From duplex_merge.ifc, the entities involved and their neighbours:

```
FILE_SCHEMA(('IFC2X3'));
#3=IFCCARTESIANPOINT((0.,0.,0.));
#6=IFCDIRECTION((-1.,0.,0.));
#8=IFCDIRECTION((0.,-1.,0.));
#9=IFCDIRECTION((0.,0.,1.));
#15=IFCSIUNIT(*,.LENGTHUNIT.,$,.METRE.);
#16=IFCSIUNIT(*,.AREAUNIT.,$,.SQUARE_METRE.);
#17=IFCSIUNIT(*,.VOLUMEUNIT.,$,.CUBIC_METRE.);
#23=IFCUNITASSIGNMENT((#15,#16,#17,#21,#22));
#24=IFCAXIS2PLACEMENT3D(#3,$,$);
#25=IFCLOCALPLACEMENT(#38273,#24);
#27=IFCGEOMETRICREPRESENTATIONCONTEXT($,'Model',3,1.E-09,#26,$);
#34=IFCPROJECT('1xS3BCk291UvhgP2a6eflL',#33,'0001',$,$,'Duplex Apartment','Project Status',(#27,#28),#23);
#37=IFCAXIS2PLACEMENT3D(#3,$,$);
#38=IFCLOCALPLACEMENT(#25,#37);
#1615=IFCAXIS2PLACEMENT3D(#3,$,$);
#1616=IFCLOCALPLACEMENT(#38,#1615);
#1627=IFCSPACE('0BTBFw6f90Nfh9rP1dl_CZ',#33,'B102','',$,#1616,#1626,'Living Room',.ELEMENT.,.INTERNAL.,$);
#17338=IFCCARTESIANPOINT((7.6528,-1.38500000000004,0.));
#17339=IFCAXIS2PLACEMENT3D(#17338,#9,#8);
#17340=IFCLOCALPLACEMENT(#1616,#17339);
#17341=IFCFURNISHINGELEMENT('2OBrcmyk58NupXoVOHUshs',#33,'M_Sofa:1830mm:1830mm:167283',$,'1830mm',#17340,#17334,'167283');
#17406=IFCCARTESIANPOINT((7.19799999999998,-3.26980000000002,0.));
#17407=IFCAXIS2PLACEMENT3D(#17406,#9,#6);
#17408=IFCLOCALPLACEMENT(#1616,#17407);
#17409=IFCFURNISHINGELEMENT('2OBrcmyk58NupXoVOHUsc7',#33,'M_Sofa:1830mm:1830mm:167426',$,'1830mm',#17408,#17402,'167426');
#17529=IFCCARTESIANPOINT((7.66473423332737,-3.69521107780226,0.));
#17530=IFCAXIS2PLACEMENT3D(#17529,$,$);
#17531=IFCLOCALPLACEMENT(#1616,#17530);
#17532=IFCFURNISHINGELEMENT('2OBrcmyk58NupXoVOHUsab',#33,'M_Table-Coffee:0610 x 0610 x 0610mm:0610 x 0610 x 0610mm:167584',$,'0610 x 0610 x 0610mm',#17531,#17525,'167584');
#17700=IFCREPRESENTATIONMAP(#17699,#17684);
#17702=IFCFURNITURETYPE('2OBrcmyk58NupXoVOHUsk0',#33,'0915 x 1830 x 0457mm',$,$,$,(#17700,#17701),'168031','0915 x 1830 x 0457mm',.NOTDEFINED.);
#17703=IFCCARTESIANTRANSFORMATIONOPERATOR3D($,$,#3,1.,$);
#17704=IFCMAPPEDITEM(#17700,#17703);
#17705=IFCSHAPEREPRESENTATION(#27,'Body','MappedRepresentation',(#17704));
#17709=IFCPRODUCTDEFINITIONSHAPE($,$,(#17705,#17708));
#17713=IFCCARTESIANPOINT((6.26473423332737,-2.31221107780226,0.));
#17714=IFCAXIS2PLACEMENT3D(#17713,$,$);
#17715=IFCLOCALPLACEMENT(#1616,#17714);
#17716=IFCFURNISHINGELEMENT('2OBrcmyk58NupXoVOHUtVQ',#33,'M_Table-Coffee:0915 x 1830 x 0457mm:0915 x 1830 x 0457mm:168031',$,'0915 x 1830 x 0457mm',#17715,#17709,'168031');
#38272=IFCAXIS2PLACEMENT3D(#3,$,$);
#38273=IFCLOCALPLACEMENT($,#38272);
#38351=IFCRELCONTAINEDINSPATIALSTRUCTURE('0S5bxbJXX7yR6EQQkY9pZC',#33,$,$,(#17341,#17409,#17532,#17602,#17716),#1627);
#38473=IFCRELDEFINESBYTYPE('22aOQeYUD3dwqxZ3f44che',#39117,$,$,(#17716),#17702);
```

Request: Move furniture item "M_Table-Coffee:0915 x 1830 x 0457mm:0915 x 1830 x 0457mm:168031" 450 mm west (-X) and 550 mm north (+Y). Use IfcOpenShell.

```python
import ifcopenshell
import ifcopenshell.api.geometry
import ifcopenshell.util.placement
import ifcopenshell.util.unit

model = ifcopenshell.open("duplex_merge.ifc")
unit_scale = ifcopenshell.util.unit.calculate_unit_scale(model)

item = model.by_guid("2OBrcmyk58NupXoVOHUtVQ")
matrix = ifcopenshell.util.placement.get_local_placement(item.ObjectPlacement)
matrix[0, 3] -= 0.45 / unit_scale
matrix[1, 3] += 0.55 / unit_scale
ifcopenshell.api.geometry.edit_object_placement(model, product=item, matrix=matrix, is_si=False)

print(ifcopenshell.util.placement.get_local_placement(item.ObjectPlacement).round(3) + 0.0)

model.write("duplex_merge-out.ifc")
```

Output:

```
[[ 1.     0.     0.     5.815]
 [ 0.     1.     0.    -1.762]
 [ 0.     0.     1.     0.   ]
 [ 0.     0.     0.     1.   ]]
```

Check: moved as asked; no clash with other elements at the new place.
